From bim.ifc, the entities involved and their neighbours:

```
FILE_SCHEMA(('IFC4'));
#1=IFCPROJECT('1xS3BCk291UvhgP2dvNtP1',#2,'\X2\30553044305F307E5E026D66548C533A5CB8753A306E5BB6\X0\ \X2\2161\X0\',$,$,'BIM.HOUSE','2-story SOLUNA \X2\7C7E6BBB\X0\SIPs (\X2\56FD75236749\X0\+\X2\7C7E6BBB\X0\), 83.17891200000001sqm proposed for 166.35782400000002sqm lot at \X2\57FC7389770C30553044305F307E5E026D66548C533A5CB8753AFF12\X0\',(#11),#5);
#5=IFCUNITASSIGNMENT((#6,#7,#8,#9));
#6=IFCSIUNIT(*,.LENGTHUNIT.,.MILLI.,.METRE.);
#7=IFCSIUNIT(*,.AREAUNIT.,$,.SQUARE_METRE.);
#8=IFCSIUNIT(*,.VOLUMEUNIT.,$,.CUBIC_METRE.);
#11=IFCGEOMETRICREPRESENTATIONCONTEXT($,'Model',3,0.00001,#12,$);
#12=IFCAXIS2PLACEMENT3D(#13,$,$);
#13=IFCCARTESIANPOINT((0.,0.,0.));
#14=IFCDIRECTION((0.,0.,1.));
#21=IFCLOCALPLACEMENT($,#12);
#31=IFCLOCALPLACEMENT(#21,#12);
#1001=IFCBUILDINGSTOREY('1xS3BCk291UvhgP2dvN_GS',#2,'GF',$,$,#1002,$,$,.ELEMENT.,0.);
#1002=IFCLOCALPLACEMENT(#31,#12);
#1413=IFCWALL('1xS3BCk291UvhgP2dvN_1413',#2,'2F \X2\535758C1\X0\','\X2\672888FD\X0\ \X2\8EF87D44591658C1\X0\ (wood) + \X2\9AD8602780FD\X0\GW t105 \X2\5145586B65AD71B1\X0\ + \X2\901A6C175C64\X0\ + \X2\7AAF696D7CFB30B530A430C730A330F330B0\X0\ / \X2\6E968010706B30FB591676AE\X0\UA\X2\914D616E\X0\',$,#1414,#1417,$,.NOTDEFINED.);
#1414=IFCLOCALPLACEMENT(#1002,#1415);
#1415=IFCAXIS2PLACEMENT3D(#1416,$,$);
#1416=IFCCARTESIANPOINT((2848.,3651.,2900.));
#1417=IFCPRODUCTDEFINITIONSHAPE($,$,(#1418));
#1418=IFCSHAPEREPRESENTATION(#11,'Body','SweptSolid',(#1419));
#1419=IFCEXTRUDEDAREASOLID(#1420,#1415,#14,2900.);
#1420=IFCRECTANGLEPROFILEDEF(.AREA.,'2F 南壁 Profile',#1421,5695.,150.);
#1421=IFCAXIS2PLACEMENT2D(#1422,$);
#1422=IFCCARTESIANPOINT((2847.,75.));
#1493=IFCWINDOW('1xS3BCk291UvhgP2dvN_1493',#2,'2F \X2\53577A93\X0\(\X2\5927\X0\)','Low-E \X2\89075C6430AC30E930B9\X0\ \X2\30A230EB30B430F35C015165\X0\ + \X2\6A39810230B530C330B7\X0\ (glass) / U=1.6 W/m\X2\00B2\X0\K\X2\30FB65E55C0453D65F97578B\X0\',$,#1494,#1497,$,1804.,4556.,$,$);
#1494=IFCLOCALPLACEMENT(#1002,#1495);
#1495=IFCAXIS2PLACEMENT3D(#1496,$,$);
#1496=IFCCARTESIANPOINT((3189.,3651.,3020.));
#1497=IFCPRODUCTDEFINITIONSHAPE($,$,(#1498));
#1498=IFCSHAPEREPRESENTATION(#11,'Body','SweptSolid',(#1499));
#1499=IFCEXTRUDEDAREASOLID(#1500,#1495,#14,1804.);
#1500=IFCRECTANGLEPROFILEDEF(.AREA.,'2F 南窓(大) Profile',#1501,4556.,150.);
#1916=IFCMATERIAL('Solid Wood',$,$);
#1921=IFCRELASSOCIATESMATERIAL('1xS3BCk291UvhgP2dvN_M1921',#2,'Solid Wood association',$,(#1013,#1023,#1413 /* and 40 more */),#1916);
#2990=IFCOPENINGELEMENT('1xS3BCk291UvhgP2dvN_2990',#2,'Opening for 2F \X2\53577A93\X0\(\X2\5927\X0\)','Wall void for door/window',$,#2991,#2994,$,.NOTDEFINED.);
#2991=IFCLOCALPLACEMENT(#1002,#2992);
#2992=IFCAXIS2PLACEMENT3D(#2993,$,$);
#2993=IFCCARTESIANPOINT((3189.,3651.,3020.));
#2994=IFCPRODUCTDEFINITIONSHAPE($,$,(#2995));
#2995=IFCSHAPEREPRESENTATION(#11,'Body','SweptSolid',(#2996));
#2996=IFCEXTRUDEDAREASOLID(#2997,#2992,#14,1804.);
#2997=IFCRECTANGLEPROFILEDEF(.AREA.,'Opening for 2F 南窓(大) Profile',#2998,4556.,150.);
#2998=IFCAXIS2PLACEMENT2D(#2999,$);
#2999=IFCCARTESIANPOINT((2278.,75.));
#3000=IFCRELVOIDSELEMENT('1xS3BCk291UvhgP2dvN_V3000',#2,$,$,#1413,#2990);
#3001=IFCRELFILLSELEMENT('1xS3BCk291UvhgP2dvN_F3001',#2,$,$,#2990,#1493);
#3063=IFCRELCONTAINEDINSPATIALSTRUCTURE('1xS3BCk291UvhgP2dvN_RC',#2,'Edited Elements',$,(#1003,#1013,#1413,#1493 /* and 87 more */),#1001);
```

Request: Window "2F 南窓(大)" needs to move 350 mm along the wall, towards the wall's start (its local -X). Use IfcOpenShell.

```python
import ifcopenshell
import ifcopenshell.api.geometry
import ifcopenshell.util.placement

model = ifcopenshell.open("bim.ifc")

window = model.by_guid("1xS3BCk291UvhgP2dvN_1493")
opening = window.FillsVoids[0].RelatingOpeningElement
wall = opening.VoidsElements[0].RelatingBuildingElement

wall_matrix = ifcopenshell.util.placement.get_local_placement(wall.ObjectPlacement)
shift = wall_matrix[:3, 0] * -350.0
before = ifcopenshell.util.placement.get_local_placement(window.ObjectPlacement)[:3, 3].copy()

# The window is not placed relative to its opening, so move both.
for product in (opening, window):
    matrix = ifcopenshell.util.placement.get_local_placement(product.ObjectPlacement)
    matrix[:3, 3] += shift
    ifcopenshell.api.geometry.edit_object_placement(model, product=product, matrix=matrix, is_si=False)

after = ifcopenshell.util.placement.get_local_placement(window.ObjectPlacement)[:3, 3]
print("window moved by", (after - before).round(3) + 0.0)

model.write("bim_v2.ifc")
```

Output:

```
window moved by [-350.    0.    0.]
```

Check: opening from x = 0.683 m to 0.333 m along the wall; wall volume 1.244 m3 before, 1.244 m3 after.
